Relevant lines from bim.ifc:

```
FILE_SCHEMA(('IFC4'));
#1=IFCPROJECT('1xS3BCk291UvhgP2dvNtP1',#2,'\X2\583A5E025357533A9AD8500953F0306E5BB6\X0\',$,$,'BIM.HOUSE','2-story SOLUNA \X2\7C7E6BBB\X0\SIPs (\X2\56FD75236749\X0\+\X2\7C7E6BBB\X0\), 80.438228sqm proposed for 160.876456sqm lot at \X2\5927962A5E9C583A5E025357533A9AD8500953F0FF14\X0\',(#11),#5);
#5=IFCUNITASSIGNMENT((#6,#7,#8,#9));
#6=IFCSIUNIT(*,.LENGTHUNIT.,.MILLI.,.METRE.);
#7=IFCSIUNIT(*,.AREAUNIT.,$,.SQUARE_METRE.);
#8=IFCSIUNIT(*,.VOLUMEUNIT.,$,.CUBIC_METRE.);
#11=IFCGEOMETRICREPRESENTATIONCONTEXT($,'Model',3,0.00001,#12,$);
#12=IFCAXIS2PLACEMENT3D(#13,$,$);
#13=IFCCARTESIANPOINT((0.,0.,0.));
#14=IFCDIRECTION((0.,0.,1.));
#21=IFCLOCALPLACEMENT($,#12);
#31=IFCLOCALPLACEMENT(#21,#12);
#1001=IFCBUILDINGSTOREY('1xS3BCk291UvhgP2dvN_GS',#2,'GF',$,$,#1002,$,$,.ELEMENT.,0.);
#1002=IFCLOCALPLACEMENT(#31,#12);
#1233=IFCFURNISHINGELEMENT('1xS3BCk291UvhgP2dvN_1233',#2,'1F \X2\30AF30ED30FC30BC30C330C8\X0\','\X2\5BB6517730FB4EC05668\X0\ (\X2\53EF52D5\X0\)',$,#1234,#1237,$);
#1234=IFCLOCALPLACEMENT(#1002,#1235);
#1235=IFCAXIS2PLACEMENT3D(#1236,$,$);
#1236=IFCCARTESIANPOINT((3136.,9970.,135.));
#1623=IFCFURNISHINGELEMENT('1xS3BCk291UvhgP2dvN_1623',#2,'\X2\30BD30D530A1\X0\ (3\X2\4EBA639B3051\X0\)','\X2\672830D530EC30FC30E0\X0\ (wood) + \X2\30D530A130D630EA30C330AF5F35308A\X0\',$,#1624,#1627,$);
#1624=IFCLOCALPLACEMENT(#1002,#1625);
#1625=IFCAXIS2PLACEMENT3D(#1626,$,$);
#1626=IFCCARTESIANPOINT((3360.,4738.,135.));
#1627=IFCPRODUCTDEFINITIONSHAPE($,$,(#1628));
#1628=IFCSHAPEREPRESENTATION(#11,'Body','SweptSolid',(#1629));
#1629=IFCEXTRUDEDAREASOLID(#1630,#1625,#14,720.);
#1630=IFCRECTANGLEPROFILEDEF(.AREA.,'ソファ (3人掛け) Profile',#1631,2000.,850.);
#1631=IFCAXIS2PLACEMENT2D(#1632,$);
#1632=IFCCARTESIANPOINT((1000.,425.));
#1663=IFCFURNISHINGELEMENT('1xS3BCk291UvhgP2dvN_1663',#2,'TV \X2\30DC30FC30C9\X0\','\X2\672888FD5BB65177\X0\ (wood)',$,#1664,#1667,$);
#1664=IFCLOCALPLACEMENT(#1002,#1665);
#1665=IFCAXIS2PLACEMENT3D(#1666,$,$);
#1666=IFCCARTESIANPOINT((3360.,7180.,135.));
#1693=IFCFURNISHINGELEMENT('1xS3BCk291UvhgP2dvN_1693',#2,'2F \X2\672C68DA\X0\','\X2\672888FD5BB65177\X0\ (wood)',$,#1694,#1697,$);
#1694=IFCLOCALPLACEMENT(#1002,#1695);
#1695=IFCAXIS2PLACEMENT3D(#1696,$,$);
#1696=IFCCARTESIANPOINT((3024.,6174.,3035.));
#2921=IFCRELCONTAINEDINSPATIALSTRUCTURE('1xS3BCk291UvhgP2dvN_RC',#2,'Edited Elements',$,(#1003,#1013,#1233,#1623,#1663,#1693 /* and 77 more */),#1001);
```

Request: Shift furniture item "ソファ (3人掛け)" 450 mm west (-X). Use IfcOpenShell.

```python
import ifcopenshell
import ifcopenshell.api.geometry
import ifcopenshell.util.placement
import ifcopenshell.util.unit

model = ifcopenshell.open("bim.ifc")
unit_scale = ifcopenshell.util.unit.calculate_unit_scale(model)

item = model.by_id(1623)
matrix = ifcopenshell.util.placement.get_local_placement(item.ObjectPlacement)
matrix[0, 3] -= 0.45 / unit_scale
ifcopenshell.api.geometry.edit_object_placement(model, product=item, matrix=matrix, is_si=False)

print(ifcopenshell.util.placement.get_local_placement(item.ObjectPlacement).round(3) + 0.0)

model.write("bim-out.ifc")
```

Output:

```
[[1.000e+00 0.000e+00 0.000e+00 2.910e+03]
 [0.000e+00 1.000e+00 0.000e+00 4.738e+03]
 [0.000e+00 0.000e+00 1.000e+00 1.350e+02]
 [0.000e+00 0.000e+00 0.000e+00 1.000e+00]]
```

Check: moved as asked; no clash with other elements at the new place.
